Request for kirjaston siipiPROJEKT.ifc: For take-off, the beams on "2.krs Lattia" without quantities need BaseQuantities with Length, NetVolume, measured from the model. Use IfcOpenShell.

First a look at what the model holds.

```python
import ifcopenshell
import ifcopenshell.util.element
import ifcopenshell.util.unit

model = ifcopenshell.open("kirjaston siipiPROJEKT.ifc")
print(model.schema)
for unit_type in ("LENGTHUNIT", "AREAUNIT", "VOLUMEUNIT"):
    print(unit_type, ifcopenshell.util.unit.calculate_unit_scale(model, unit_type))
storey = next(s for s in model.by_type("IfcBuildingStorey") if s.Name == "2.krs Lattia")
beams = [e for e in ifcopenshell.util.element.get_decomposition(storey) if e.is_a("IfcBeam")]
for e in sorted(beams, key=lambda e: e.id()):
    print(e.id(), e.is_a(), e.Name, list(ifcopenshell.util.element.get_psets(e, qtos_only=True)), sep=" | ")
```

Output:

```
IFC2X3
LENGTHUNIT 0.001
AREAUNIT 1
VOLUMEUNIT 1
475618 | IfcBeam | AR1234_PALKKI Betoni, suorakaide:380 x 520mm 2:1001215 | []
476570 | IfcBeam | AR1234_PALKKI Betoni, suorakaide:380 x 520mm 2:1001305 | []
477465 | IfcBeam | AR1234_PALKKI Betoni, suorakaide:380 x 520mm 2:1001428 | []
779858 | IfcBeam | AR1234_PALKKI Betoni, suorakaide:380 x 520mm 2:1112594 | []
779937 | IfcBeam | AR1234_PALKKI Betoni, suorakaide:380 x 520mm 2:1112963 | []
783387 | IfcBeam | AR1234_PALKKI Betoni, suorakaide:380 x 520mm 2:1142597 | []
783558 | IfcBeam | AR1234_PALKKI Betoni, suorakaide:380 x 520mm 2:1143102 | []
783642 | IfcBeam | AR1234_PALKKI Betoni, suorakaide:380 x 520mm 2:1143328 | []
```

```python
import ifcopenshell
import ifcopenshell.api.pset
import ifcopenshell.geom
import ifcopenshell.util.element
import ifcopenshell.util.shape
import ifcopenshell.util.unit

model = ifcopenshell.open("kirjaston siipiPROJEKT.ifc")
unit_scale = ifcopenshell.util.unit.calculate_unit_scale(model)
volume_scale = ifcopenshell.util.unit.calculate_unit_scale(model, "VOLUMEUNIT")
settings = ifcopenshell.geom.settings()

storey = next(s for s in model.by_type("IfcBuildingStorey") if s.Name == "2.krs Lattia")
beams = [e for e in ifcopenshell.util.element.get_decomposition(storey) if e.is_a("IfcBeam")]

for e in sorted(beams, key=lambda e: e.id()):
    if ifcopenshell.util.element.get_psets(e, qtos_only=True, should_inherit=False):
        continue
    # Geometry comes back in metres, in the element's own axes.
    shape = ifcopenshell.geom.create_shape(settings, e)
    values = {
        "Length": ifcopenshell.util.shape.get_max_xyz(shape.geometry) / unit_scale,
        "NetVolume": ifcopenshell.util.shape.get_volume(shape.geometry) / volume_scale,
    }
    qto = ifcopenshell.api.pset.add_qto(model, product=e, name="BaseQuantities")
    ifcopenshell.api.pset.edit_qto(model, qto=qto, properties=values)
    print(e.id(), {k: round(v, 3) for k, v in values.items()})

model.write("kirjaston siipiPROJEKT_v2.ifc")
```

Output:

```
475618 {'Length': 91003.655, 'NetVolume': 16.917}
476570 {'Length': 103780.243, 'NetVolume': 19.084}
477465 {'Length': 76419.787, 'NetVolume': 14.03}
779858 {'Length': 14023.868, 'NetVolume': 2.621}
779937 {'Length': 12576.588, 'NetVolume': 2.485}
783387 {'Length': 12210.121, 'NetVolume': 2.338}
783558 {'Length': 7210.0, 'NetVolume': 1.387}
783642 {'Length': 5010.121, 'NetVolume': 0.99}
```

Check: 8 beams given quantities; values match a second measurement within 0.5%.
